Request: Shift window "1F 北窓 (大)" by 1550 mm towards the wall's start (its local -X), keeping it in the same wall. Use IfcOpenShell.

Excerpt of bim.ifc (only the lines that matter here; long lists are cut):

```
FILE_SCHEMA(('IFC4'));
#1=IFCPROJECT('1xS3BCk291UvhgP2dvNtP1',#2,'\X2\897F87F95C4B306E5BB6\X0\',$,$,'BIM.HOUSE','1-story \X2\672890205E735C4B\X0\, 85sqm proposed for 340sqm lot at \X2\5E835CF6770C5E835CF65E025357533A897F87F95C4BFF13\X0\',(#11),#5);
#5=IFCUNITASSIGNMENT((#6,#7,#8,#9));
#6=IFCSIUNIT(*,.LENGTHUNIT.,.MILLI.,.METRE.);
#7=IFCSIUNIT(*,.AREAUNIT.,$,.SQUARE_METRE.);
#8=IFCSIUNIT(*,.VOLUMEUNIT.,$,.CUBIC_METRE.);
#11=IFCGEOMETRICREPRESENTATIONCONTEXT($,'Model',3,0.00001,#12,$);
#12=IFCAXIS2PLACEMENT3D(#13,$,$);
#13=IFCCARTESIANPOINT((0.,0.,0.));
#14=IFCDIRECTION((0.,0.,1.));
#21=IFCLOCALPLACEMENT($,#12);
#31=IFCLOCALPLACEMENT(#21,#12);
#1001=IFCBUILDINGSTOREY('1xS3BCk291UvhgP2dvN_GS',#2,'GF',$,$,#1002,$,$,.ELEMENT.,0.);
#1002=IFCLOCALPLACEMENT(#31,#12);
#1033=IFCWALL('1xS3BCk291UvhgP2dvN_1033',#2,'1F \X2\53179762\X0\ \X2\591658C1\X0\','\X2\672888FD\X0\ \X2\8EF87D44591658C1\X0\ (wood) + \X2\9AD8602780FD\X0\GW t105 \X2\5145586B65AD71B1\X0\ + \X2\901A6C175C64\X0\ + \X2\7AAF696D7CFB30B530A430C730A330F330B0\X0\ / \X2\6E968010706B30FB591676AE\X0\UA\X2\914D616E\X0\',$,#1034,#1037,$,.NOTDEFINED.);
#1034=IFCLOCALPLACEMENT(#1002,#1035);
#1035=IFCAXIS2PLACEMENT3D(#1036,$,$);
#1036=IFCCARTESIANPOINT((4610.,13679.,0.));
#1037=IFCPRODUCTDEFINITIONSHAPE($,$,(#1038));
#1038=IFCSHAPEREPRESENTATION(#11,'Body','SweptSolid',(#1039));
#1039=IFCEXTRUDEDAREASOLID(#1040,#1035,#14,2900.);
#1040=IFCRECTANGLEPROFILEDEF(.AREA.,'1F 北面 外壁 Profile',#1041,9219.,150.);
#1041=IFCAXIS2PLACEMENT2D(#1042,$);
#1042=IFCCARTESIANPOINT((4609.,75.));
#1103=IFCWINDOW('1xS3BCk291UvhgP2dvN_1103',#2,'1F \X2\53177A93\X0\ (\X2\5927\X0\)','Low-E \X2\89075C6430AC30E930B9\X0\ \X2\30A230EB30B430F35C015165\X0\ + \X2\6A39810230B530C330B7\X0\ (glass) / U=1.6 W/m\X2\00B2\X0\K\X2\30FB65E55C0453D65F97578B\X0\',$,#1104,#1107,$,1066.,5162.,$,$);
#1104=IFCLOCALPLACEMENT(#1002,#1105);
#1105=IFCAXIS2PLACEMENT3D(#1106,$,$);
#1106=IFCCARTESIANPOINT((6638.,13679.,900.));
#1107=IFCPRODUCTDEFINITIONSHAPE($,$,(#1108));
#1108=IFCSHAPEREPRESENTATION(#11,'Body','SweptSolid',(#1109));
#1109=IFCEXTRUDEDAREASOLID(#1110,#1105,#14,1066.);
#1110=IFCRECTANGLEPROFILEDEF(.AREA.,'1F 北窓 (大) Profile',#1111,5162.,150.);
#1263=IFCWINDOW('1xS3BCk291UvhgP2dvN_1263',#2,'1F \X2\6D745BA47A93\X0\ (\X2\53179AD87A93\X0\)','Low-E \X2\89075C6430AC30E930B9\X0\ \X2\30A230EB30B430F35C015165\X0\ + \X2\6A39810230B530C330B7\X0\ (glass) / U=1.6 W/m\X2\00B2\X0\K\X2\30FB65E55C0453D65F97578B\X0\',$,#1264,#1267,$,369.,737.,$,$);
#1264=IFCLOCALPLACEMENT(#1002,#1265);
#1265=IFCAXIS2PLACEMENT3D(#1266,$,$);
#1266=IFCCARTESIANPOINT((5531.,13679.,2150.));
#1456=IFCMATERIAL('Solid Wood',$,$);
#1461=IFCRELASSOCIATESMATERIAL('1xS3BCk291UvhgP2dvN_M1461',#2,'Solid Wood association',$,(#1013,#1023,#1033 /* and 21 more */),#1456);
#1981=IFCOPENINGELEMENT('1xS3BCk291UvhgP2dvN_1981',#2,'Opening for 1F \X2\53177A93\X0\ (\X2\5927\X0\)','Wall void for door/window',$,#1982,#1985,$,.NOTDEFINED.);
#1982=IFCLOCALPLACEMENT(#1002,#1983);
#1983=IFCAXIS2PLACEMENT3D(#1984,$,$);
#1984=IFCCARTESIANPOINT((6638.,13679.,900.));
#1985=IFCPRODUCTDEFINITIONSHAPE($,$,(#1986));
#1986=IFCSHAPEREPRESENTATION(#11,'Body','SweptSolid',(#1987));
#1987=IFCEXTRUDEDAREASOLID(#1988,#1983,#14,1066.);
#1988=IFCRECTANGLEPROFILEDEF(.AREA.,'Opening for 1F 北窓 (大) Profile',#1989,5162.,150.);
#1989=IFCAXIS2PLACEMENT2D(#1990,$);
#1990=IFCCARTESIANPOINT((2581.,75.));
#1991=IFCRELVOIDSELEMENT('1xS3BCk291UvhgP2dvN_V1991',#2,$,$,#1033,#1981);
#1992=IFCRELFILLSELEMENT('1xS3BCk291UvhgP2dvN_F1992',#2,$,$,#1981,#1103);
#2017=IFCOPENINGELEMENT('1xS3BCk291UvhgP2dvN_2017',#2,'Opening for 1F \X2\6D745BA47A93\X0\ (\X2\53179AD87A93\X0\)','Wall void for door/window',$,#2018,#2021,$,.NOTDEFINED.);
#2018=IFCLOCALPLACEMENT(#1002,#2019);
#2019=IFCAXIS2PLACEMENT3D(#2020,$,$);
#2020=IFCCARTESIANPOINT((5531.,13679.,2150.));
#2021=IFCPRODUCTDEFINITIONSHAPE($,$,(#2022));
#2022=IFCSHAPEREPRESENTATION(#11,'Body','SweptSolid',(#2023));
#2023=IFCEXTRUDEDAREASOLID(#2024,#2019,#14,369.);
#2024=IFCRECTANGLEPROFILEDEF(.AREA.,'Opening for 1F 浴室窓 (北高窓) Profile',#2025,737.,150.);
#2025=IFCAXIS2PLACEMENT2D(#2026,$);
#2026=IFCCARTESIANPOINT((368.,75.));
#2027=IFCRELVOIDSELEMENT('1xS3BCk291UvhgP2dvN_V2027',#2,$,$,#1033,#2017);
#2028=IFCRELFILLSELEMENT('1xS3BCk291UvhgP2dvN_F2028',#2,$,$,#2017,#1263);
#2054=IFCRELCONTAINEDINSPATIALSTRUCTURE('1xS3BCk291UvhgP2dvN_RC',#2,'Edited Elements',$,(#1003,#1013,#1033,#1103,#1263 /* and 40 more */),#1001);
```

```python
import ifcopenshell
import ifcopenshell.api.geometry
import ifcopenshell.util.placement

model = ifcopenshell.open("bim.ifc")

window = model.by_guid("1xS3BCk291UvhgP2dvN_1103")
opening = window.FillsVoids[0].RelatingOpeningElement
wall = opening.VoidsElements[0].RelatingBuildingElement

wall_matrix = ifcopenshell.util.placement.get_local_placement(wall.ObjectPlacement)
shift = wall_matrix[:3, 0] * -1550.0
before = ifcopenshell.util.placement.get_local_placement(window.ObjectPlacement)[:3, 3].copy()

# The window is not placed relative to its opening, so move both.
for product in (opening, window):
    matrix = ifcopenshell.util.placement.get_local_placement(product.ObjectPlacement)
    matrix[:3, 3] += shift
    ifcopenshell.api.geometry.edit_object_placement(model, product=product, matrix=matrix, is_si=False)

after = ifcopenshell.util.placement.get_local_placement(window.ObjectPlacement)[:3, 3]
print("window moved by", (after - before).round(3) + 0.0)

model.write("bim_edited.ifc")
```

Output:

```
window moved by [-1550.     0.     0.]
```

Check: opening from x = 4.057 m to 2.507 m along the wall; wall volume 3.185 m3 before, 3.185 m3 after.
